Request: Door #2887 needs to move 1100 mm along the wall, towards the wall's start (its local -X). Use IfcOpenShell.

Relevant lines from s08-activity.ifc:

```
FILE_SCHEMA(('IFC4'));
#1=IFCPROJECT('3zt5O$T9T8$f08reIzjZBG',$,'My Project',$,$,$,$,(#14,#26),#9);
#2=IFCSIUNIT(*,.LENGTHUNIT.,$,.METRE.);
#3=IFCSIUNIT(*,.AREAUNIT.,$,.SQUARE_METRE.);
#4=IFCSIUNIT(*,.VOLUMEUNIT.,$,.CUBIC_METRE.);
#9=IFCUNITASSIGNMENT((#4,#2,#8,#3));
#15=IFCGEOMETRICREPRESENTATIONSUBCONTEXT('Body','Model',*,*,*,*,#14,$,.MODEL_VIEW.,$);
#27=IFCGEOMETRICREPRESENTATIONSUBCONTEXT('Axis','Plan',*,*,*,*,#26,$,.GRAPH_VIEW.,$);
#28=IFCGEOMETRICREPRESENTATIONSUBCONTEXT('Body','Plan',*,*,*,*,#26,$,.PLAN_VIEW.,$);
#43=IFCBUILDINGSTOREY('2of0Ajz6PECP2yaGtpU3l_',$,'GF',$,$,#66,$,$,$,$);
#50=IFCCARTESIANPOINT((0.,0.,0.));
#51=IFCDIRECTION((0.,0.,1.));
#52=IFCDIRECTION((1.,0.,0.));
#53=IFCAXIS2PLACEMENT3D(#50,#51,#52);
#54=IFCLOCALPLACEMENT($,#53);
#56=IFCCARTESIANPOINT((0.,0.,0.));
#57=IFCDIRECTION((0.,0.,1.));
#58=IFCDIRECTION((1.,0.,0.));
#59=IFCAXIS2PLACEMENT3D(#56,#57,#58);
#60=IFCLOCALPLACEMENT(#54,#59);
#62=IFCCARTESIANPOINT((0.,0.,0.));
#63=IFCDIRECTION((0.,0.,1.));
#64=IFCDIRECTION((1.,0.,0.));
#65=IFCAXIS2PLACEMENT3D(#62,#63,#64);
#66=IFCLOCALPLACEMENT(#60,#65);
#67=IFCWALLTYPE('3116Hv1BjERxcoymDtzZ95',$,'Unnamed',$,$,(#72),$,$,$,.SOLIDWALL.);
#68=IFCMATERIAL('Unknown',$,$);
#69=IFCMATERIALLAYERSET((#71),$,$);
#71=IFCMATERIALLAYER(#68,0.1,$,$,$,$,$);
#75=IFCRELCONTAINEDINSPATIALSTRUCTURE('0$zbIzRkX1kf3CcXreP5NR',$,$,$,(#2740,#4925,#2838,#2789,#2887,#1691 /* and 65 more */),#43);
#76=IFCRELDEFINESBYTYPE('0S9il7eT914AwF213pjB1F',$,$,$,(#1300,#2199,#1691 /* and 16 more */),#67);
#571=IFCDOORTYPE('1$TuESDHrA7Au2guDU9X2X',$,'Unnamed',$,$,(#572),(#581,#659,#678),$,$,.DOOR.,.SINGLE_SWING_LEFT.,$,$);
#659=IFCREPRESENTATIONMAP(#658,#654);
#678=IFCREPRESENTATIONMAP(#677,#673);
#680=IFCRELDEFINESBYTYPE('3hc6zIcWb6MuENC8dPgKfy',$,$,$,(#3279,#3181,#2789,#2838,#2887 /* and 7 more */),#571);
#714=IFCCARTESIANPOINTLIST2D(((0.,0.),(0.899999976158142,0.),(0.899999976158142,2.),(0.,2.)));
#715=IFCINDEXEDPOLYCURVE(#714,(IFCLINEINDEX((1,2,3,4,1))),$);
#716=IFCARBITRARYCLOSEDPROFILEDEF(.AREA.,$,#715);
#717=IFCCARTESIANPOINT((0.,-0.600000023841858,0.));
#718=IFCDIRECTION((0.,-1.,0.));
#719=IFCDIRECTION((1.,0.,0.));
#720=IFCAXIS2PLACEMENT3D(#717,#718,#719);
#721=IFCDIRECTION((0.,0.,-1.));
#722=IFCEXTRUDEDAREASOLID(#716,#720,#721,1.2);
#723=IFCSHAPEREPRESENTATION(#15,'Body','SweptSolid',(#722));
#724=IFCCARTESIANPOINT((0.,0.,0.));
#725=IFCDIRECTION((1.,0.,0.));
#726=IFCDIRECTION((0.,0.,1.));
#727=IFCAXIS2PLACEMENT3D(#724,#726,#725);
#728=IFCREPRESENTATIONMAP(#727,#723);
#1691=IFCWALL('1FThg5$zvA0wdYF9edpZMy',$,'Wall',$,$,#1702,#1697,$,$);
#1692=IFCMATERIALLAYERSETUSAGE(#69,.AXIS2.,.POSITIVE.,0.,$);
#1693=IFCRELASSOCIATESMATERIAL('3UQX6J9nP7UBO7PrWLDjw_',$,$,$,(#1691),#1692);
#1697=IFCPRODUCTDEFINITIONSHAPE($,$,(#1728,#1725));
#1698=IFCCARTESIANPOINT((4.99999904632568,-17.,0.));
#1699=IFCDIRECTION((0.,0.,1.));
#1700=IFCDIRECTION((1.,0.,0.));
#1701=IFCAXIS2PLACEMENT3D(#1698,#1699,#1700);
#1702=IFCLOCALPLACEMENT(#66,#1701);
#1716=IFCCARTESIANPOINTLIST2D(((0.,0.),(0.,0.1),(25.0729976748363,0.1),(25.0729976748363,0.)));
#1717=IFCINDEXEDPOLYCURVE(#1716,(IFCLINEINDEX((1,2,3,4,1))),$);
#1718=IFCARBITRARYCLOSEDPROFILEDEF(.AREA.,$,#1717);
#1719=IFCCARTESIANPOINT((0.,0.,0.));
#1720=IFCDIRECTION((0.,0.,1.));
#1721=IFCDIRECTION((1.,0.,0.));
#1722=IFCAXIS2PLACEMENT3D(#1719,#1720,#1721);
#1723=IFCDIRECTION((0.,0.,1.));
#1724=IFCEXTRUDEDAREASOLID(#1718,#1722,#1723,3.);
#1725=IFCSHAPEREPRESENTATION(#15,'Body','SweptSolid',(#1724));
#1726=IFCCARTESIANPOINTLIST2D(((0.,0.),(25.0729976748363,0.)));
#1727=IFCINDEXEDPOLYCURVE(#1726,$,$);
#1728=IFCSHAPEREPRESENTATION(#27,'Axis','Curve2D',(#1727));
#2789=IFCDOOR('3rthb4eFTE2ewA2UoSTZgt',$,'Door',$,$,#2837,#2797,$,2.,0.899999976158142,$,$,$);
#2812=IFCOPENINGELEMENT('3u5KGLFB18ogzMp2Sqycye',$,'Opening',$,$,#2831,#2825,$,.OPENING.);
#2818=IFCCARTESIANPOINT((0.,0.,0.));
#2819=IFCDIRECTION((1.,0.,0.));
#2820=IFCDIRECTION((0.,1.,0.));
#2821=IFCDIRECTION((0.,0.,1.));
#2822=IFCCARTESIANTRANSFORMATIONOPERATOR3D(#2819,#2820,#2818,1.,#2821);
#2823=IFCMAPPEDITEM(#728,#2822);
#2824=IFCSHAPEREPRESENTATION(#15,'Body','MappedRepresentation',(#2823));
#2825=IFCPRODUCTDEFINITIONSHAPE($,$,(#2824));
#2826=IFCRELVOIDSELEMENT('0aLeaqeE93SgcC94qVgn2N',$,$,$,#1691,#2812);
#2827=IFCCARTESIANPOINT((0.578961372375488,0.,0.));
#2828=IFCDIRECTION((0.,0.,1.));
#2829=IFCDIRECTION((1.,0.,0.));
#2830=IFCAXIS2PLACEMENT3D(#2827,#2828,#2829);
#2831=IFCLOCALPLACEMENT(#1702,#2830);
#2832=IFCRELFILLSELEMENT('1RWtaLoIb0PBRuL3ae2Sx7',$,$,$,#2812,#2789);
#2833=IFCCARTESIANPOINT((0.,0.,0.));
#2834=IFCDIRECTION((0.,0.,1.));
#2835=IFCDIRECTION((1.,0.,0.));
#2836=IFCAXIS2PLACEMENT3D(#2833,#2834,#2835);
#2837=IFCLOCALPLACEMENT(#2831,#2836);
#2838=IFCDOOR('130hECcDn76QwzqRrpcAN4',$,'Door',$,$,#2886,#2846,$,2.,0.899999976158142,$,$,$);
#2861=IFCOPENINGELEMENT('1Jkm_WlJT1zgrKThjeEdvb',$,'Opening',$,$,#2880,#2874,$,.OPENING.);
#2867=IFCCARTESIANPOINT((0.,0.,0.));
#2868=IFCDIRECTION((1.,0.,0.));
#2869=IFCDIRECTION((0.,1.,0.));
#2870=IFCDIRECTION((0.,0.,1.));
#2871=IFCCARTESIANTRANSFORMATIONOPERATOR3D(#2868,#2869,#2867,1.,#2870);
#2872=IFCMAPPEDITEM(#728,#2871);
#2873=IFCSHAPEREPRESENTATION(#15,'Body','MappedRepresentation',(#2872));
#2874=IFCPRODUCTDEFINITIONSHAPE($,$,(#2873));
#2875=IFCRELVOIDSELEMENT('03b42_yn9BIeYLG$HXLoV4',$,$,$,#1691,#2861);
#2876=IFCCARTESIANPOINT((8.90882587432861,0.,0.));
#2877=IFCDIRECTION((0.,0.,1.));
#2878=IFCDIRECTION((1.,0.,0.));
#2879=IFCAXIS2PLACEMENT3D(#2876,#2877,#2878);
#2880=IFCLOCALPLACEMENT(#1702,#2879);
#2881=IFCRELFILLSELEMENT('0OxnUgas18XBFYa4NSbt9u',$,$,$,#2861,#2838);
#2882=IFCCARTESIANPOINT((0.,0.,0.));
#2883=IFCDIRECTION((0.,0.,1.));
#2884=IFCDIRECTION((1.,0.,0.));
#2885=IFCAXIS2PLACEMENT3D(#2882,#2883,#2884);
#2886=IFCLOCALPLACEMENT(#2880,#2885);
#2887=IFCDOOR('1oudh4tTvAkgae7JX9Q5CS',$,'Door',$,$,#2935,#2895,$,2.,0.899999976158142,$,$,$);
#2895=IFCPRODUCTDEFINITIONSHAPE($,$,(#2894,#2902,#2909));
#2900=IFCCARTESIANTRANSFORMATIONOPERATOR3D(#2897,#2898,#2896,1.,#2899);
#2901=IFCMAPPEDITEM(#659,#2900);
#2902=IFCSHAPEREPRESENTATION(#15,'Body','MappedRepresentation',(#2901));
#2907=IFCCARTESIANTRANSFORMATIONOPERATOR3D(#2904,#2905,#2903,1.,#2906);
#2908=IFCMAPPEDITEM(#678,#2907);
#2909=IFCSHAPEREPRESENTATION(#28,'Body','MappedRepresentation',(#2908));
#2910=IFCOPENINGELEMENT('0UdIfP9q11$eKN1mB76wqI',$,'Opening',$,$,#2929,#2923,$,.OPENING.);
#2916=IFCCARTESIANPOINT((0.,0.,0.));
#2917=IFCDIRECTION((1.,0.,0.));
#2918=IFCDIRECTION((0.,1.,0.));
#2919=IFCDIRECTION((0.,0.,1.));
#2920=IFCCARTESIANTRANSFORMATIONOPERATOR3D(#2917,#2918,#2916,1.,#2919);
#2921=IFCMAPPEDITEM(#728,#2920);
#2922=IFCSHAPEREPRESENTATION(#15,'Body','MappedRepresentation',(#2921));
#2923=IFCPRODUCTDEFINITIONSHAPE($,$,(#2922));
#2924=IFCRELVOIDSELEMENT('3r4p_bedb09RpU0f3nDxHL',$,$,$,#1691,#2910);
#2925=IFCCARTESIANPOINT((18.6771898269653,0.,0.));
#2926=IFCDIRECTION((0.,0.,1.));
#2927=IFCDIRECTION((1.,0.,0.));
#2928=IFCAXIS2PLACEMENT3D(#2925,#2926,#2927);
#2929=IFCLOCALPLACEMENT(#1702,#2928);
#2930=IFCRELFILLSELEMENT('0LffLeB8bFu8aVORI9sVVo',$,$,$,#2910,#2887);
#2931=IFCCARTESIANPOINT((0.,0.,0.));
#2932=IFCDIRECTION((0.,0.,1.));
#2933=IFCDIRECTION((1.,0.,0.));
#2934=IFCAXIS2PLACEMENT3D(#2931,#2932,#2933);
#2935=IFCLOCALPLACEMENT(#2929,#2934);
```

```python
import ifcopenshell
import ifcopenshell.api.geometry
import ifcopenshell.util.placement
import ifcopenshell.util.unit

model = ifcopenshell.open("s08-activity.ifc")
unit_scale = ifcopenshell.util.unit.calculate_unit_scale(model)

door = model.by_guid("1oudh4tTvAkgae7JX9Q5CS")
opening = door.FillsVoids[0].RelatingOpeningElement
wall = opening.VoidsElements[0].RelatingBuildingElement

wall_matrix = ifcopenshell.util.placement.get_local_placement(wall.ObjectPlacement)
shift = wall_matrix[:3, 0] * -1.1 / unit_scale
before = ifcopenshell.util.placement.get_local_placement(door.ObjectPlacement)[:3, 3].copy()

# The door is placed relative to its opening, so it follows when the opening moves.
matrix = ifcopenshell.util.placement.get_local_placement(opening.ObjectPlacement)
matrix[:3, 3] += shift
ifcopenshell.api.geometry.edit_object_placement(
    model, product=opening, matrix=matrix, is_si=False, should_transform_children=True
)

after = ifcopenshell.util.placement.get_local_placement(door.ObjectPlacement)[:3, 3]
print("door moved by", (after - before).round(3) + 0.0)

model.write("s08-activity_edited.ifc")
```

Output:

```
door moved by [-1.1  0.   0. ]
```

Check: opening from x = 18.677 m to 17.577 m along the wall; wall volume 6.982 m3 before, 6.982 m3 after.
